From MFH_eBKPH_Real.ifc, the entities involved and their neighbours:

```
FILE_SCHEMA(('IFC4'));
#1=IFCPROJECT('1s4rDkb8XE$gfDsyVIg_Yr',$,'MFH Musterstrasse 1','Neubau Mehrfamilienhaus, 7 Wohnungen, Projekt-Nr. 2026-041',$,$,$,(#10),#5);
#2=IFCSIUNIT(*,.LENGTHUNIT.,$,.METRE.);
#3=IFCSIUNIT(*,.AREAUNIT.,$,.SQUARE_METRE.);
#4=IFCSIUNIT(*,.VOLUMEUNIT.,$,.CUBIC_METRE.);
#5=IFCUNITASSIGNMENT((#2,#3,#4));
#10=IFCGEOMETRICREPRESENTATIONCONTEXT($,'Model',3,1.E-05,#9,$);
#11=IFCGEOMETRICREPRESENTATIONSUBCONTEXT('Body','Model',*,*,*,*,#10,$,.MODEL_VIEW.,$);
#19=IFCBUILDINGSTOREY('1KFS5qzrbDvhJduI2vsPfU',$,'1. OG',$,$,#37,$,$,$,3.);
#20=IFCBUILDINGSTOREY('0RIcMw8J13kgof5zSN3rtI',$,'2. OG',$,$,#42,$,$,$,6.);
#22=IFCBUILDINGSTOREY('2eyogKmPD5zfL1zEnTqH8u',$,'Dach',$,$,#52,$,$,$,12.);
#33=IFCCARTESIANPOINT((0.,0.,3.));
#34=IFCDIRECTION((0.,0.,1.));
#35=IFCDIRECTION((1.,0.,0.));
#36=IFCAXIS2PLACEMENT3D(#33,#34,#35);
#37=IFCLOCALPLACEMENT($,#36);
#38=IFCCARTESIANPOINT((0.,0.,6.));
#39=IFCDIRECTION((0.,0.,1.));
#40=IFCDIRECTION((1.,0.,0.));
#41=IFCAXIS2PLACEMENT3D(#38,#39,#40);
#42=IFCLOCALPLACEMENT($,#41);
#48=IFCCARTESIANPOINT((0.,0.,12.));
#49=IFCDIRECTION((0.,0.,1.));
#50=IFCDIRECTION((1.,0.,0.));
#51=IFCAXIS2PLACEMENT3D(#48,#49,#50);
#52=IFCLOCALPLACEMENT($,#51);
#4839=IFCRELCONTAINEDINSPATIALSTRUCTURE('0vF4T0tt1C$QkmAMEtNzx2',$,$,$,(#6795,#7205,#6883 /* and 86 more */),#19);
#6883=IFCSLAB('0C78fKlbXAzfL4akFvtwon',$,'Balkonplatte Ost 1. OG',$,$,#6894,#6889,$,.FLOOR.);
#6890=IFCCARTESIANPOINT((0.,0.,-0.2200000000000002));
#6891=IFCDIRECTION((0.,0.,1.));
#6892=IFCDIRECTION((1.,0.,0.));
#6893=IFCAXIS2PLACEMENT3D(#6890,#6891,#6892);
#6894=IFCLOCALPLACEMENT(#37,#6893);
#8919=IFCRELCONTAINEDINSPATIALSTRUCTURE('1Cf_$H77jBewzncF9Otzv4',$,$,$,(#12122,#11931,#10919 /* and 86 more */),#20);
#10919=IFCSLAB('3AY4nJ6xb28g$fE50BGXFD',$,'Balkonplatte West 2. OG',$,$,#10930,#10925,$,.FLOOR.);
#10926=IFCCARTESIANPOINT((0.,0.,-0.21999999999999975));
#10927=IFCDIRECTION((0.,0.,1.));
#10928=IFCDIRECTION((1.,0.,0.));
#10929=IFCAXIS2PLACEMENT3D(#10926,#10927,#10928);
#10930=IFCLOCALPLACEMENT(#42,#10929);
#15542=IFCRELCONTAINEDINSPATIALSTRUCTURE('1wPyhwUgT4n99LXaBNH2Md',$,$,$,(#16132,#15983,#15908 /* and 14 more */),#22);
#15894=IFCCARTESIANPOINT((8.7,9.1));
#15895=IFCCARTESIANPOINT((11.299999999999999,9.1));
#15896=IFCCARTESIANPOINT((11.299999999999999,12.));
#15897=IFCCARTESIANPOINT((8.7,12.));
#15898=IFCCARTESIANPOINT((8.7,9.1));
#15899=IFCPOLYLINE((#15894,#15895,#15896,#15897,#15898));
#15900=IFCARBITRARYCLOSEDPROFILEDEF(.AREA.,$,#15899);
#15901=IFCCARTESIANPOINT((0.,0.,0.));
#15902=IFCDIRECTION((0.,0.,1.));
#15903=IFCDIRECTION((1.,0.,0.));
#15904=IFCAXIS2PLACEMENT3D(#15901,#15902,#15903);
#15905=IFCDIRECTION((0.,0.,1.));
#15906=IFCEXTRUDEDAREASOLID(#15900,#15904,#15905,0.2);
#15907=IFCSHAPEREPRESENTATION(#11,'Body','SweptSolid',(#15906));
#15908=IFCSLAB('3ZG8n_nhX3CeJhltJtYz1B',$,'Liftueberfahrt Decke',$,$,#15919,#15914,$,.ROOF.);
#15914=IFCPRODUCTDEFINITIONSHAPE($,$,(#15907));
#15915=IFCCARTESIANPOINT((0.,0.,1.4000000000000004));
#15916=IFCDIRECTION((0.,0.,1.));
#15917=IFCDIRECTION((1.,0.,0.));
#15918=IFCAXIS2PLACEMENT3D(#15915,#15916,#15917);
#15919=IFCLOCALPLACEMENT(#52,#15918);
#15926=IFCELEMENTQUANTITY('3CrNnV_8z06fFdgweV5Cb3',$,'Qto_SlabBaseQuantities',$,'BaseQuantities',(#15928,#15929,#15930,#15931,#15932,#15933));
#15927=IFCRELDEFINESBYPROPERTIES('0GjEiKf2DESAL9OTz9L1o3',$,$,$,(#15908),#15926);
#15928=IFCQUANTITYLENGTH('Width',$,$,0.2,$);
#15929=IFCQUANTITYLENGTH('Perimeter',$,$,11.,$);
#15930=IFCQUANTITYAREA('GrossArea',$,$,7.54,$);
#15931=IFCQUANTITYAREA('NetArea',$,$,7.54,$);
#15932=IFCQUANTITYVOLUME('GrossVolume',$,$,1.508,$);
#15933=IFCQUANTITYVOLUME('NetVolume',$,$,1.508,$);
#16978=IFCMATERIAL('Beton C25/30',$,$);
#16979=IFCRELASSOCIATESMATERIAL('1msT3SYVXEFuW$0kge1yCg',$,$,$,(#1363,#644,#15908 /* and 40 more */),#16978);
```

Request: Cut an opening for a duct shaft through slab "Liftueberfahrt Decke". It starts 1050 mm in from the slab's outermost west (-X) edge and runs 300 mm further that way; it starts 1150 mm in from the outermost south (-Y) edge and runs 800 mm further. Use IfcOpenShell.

```python
import numpy as np
import ifcopenshell
import ifcopenshell.api.feature
import ifcopenshell.api.geometry
import ifcopenshell.api.pset
import ifcopenshell.api.root
import ifcopenshell.geom
import ifcopenshell.util.element
import ifcopenshell.util.placement
import ifcopenshell.util.representation
import ifcopenshell.util.shape
import ifcopenshell.util.unit

model = ifcopenshell.open("MFH_eBKPH_Real.ifc")
unit_scale = ifcopenshell.util.unit.calculate_unit_scale(model)
area_scale = ifcopenshell.util.unit.calculate_unit_scale(model, "AREAUNIT")
volume_scale = ifcopenshell.util.unit.calculate_unit_scale(model, "VOLUMEUNIT")
settings = ifcopenshell.geom.settings()


def volume(element):
    """Net volume in cubic metres, openings subtracted."""
    shape = ifcopenshell.geom.create_shape(settings, element)
    return ifcopenshell.util.shape.get_volume(shape.geometry)


slab = model.by_guid("3ZG8n_nhX3CeJhltJtYz1B")
before = volume(slab)

# Extent in the slab's own axes, in metres. The edges named are its -X and -Y sides.
slab_shape = ifcopenshell.geom.create_shape(settings, slab)
vertices = ifcopenshell.util.shape.get_vertices(slab_shape.geometry)
x_min, y_min, bottom = vertices.min(axis=0)
top = vertices[:, 2].max()

opening = ifcopenshell.api.root.create_entity(model, ifc_class="IfcOpeningElement", name="Duct shaft opening", predefined_type="OPENING")
context = ifcopenshell.util.representation.get_context(model, "Model", "Body", "MODEL_VIEW")
width, depth = 0.3, 0.8
outline = [(0.0, 0.0), (width, 0.0), (width, depth), (0.0, depth), (0.0, 0.0)]
# Overshoot both faces by 50 mm so the cut is clean.
shape = ifcopenshell.api.geometry.add_slab_representation(
    model, context=context, depth=top - bottom + 0.1, polyline=outline
)
ifcopenshell.api.geometry.assign_representation(model, product=opening, representation=shape)

matrix = ifcopenshell.util.placement.get_local_placement(slab.ObjectPlacement)
matrix[:, 3] = matrix @ np.append(np.array([x_min + 1.05, y_min + 1.15, bottom - 0.05]) / unit_scale, 1.0)
ifcopenshell.api.geometry.edit_object_placement(model, product=opening, matrix=matrix, is_si=False)
ifcopenshell.api.feature.add_feature(model, feature=opening, element=slab)

after = volume(slab)

# Update the slab's stored quantities.
qto = model.by_id(ifcopenshell.util.element.get_pset(slab, "Qto_SlabBaseQuantities", should_inherit=False)["id"])
ifcopenshell.api.pset.edit_qto(model, qto=qto, properties={
    "NetArea": after / (top - bottom) / area_scale,
    "NetVolume": after / volume_scale,
})

print(f"slab volume {before:.3f} -> {after:.3f} m3")

model.write("MFH_eBKPH_Real_rev.ifc")
```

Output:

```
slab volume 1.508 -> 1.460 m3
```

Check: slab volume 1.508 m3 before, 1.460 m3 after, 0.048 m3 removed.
